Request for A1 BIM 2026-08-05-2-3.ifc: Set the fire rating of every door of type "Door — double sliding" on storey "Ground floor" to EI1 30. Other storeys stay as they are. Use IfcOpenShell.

First a look at what the model holds.

```python
import ifcopenshell
import ifcopenshell.util.element

model = ifcopenshell.open("A1 BIM 2026-08-05-2-3.ifc")
print(model.schema)
storey = next(s for s in model.by_type("IfcBuildingStorey") if s.Name == "Ground floor")
doors = [e for e in ifcopenshell.util.element.get_decomposition(storey) if e.is_a("IfcDoor")]
seen = {}
for e in doors:
    element_type = ifcopenshell.util.element.get_type(e)
    key = (element_type.Name if element_type != e and element_type else None, ifcopenshell.util.element.get_pset(e, "Pset_DoorCommon", "FireRating"))
    seen[key] = seen.get(key, 0) + 1
for (name, value), count in sorted(seen.items(), key=str):
    print(count, "x", name, "|", value)
```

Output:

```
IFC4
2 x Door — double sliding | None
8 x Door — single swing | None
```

```python
import ifcopenshell
import ifcopenshell.api.pset
import ifcopenshell.util.element

model = ifcopenshell.open("A1 BIM 2026-08-05-2-3.ifc")

storey = next(s for s in model.by_type("IfcBuildingStorey") if s.Name == "Ground floor")
doors = [e for e in ifcopenshell.util.element.get_decomposition(storey) if e.is_a("IfcDoor")]

count = 0
for e in doors:
    element_type = ifcopenshell.util.element.get_type(e)
    if element_type in (None, e) or element_type.Name != "Door — double sliding":
        continue
    # add_pset returns the element's existing set when there is one.
    pset = ifcopenshell.api.pset.add_pset(model, product=e, name="Pset_DoorCommon")
    ifcopenshell.api.pset.edit_pset(model, pset=pset, properties={"FireRating": "EI1 30"})
    count += 1

print(count, "doors updated")

model.write("A1 BIM 2026-08-05-2-3-out.ifc")
```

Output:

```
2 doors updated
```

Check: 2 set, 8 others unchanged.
